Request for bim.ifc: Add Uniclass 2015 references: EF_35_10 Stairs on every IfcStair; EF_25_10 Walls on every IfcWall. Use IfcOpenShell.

First a look at what the model holds.

```python
import ifcopenshell

model = ifcopenshell.open("bim.ifc")
print(model.schema)
print("classifications:", [c.Name for c in model.by_type("IfcClassification")])
for ifc_class in ("IfcDoor", "IfcRoof", "IfcStair", "IfcWall", "IfcWindow"):
    print(ifc_class, len(model.by_type(ifc_class)))
```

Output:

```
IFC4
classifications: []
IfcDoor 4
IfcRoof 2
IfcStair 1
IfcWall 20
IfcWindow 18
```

```python
import ifcopenshell
import ifcopenshell.api.classification

model = ifcopenshell.open("bim.ifc")

system = ifcopenshell.api.classification.add_classification(model, classification="Uniclass 2015")

codes = {
    "IfcStair": ("EF_35_10", "Stairs"),
    "IfcWall": ("EF_25_10", "Walls"),
}
for ifc_class, (code, name) in codes.items():
    products = model.by_type(ifc_class)
    ifcopenshell.api.classification.add_reference(
        model, products=products, classification=system, identification=code, name=name
    )
    print(code, len(products))

model.write("bim_edited.ifc")
```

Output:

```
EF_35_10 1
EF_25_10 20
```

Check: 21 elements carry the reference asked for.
